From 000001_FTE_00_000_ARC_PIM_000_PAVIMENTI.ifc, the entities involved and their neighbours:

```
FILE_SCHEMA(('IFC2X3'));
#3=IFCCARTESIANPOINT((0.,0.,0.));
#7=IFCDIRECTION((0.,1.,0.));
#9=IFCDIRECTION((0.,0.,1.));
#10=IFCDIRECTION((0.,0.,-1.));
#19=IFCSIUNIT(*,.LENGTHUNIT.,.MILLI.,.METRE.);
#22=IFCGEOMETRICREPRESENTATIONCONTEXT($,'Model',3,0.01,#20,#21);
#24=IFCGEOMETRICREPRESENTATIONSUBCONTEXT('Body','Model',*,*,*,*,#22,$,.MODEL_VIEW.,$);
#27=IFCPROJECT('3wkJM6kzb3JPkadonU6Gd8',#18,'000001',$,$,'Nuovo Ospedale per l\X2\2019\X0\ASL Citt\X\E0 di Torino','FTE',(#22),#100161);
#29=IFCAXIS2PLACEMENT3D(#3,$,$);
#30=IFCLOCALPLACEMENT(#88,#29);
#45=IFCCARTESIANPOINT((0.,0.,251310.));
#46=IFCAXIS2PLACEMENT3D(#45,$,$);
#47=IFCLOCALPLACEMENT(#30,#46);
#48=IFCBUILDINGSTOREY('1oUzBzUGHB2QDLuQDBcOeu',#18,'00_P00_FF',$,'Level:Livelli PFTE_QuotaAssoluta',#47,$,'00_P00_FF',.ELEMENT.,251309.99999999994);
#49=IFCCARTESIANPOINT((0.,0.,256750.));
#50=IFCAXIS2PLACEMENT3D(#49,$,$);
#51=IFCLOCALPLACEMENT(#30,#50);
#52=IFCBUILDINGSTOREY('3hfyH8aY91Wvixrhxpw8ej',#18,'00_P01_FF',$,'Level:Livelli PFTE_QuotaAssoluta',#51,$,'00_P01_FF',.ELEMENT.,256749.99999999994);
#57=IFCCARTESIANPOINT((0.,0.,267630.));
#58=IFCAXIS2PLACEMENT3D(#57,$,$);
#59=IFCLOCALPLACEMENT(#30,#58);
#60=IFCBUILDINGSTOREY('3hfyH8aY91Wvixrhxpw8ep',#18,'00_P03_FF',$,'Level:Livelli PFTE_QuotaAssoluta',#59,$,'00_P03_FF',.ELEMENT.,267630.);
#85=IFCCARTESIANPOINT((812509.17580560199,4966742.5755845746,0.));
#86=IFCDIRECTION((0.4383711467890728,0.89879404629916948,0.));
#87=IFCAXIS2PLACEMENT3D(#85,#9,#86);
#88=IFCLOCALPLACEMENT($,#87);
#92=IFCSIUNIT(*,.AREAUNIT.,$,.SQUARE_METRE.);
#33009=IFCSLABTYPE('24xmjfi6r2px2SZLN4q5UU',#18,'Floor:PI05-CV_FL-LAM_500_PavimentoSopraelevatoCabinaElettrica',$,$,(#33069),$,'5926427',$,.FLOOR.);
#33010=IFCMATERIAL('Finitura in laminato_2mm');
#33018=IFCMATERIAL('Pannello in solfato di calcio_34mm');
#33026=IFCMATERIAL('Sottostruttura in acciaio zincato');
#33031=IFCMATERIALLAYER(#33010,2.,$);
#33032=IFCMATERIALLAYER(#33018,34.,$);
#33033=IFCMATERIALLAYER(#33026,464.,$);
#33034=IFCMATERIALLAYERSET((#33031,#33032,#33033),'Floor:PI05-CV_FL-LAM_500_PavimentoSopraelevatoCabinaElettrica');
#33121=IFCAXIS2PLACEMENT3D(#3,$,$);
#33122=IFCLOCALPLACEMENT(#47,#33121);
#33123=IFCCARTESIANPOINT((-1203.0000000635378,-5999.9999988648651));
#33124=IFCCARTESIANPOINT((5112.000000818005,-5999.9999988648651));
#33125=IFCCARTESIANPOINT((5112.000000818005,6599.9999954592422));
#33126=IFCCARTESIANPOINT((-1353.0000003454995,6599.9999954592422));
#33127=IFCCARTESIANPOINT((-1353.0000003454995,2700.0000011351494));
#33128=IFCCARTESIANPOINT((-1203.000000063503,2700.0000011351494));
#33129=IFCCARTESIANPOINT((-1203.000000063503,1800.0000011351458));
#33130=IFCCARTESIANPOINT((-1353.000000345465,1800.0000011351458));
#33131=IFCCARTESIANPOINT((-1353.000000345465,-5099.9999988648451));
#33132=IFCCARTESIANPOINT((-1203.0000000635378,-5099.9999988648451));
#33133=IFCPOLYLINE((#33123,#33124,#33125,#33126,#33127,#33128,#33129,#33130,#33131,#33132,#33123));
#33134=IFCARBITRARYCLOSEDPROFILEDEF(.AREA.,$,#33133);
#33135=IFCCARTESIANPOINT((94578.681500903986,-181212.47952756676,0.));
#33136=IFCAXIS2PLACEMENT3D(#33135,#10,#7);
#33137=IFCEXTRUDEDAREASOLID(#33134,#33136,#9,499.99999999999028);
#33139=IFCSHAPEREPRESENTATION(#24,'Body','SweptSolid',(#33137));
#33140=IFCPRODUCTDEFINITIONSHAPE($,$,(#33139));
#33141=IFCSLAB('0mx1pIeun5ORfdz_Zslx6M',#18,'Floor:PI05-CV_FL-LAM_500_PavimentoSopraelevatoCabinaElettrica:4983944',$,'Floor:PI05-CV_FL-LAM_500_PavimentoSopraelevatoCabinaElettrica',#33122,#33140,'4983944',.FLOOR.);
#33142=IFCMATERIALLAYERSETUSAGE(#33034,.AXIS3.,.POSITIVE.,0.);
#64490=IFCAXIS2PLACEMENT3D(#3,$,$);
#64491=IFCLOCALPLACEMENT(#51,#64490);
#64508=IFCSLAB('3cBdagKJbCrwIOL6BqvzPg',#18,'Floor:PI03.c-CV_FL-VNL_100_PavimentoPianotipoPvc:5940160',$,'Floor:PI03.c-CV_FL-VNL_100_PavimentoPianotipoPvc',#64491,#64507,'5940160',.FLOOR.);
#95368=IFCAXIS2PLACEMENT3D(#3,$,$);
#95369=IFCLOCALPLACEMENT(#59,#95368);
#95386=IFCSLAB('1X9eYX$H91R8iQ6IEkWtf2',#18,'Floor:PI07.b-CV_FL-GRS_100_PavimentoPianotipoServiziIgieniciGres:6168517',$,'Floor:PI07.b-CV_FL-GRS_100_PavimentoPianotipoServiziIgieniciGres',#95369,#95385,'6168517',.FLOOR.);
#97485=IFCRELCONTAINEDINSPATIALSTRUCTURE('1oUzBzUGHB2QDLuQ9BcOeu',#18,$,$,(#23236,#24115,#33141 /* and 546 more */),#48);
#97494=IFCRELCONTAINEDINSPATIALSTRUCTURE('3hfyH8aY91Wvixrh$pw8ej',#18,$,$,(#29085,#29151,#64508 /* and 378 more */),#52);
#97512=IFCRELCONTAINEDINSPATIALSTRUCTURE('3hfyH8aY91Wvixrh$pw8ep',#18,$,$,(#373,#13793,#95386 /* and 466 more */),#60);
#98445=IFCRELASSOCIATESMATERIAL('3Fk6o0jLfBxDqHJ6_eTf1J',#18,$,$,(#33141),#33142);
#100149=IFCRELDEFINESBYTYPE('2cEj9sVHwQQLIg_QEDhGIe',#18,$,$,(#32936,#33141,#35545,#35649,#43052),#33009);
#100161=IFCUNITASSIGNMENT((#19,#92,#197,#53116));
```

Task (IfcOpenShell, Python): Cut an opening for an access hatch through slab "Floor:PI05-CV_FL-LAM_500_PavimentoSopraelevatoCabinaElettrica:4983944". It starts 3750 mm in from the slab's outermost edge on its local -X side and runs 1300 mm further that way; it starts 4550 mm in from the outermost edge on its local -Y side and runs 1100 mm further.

```python
import numpy as np
import ifcopenshell
import ifcopenshell.api.feature
import ifcopenshell.api.geometry
import ifcopenshell.api.root
import ifcopenshell.geom
import ifcopenshell.util.placement
import ifcopenshell.util.representation
import ifcopenshell.util.shape
import ifcopenshell.util.unit

model = ifcopenshell.open("000001_FTE_00_000_ARC_PIM_000_PAVIMENTI.ifc")
unit_scale = ifcopenshell.util.unit.calculate_unit_scale(model)
settings = ifcopenshell.geom.settings()


def volume(element):
    """Net volume in cubic metres, openings subtracted."""
    shape = ifcopenshell.geom.create_shape(settings, element)
    return ifcopenshell.util.shape.get_volume(shape.geometry)


slab = model.by_guid("0mx1pIeun5ORfdz_Zslx6M")
before = volume(slab)

# Extent in the slab's own axes, in metres. The edges named are its -X and -Y sides.
slab_shape = ifcopenshell.geom.create_shape(settings, slab)
vertices = ifcopenshell.util.shape.get_vertices(slab_shape.geometry)
x_min, y_min, bottom = vertices.min(axis=0)
top = vertices[:, 2].max()

opening = ifcopenshell.api.root.create_entity(model, ifc_class="IfcOpeningElement", name="Access hatch opening")
context = ifcopenshell.util.representation.get_context(model, "Model", "Body", "MODEL_VIEW")
width, depth = 1.3, 1.1
outline = [(0.0, 0.0), (width, 0.0), (width, depth), (0.0, depth), (0.0, 0.0)]
# Overshoot both faces by 50 mm so the cut is clean.
shape = ifcopenshell.api.geometry.add_slab_representation(
    model, context=context, depth=top - bottom + 0.1, polyline=outline
)
ifcopenshell.api.geometry.assign_representation(model, product=opening, representation=shape)

matrix = ifcopenshell.util.placement.get_local_placement(slab.ObjectPlacement)
matrix[:, 3] = matrix @ np.append(np.array([x_min + 3.75, y_min + 4.55, bottom - 0.05]) / unit_scale, 1.0)
ifcopenshell.api.geometry.edit_object_placement(model, product=opening, matrix=matrix, is_si=False)
ifcopenshell.api.feature.add_feature(model, feature=opening, element=slab)

after = volume(slab)

print(f"slab volume {before:.3f} -> {after:.3f} m3")

model.write("000001_FTE_00_000_ARC_PIM_000_PAVIMENTI_edited.ifc")
```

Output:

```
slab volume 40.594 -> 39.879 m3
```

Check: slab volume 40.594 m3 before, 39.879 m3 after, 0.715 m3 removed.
